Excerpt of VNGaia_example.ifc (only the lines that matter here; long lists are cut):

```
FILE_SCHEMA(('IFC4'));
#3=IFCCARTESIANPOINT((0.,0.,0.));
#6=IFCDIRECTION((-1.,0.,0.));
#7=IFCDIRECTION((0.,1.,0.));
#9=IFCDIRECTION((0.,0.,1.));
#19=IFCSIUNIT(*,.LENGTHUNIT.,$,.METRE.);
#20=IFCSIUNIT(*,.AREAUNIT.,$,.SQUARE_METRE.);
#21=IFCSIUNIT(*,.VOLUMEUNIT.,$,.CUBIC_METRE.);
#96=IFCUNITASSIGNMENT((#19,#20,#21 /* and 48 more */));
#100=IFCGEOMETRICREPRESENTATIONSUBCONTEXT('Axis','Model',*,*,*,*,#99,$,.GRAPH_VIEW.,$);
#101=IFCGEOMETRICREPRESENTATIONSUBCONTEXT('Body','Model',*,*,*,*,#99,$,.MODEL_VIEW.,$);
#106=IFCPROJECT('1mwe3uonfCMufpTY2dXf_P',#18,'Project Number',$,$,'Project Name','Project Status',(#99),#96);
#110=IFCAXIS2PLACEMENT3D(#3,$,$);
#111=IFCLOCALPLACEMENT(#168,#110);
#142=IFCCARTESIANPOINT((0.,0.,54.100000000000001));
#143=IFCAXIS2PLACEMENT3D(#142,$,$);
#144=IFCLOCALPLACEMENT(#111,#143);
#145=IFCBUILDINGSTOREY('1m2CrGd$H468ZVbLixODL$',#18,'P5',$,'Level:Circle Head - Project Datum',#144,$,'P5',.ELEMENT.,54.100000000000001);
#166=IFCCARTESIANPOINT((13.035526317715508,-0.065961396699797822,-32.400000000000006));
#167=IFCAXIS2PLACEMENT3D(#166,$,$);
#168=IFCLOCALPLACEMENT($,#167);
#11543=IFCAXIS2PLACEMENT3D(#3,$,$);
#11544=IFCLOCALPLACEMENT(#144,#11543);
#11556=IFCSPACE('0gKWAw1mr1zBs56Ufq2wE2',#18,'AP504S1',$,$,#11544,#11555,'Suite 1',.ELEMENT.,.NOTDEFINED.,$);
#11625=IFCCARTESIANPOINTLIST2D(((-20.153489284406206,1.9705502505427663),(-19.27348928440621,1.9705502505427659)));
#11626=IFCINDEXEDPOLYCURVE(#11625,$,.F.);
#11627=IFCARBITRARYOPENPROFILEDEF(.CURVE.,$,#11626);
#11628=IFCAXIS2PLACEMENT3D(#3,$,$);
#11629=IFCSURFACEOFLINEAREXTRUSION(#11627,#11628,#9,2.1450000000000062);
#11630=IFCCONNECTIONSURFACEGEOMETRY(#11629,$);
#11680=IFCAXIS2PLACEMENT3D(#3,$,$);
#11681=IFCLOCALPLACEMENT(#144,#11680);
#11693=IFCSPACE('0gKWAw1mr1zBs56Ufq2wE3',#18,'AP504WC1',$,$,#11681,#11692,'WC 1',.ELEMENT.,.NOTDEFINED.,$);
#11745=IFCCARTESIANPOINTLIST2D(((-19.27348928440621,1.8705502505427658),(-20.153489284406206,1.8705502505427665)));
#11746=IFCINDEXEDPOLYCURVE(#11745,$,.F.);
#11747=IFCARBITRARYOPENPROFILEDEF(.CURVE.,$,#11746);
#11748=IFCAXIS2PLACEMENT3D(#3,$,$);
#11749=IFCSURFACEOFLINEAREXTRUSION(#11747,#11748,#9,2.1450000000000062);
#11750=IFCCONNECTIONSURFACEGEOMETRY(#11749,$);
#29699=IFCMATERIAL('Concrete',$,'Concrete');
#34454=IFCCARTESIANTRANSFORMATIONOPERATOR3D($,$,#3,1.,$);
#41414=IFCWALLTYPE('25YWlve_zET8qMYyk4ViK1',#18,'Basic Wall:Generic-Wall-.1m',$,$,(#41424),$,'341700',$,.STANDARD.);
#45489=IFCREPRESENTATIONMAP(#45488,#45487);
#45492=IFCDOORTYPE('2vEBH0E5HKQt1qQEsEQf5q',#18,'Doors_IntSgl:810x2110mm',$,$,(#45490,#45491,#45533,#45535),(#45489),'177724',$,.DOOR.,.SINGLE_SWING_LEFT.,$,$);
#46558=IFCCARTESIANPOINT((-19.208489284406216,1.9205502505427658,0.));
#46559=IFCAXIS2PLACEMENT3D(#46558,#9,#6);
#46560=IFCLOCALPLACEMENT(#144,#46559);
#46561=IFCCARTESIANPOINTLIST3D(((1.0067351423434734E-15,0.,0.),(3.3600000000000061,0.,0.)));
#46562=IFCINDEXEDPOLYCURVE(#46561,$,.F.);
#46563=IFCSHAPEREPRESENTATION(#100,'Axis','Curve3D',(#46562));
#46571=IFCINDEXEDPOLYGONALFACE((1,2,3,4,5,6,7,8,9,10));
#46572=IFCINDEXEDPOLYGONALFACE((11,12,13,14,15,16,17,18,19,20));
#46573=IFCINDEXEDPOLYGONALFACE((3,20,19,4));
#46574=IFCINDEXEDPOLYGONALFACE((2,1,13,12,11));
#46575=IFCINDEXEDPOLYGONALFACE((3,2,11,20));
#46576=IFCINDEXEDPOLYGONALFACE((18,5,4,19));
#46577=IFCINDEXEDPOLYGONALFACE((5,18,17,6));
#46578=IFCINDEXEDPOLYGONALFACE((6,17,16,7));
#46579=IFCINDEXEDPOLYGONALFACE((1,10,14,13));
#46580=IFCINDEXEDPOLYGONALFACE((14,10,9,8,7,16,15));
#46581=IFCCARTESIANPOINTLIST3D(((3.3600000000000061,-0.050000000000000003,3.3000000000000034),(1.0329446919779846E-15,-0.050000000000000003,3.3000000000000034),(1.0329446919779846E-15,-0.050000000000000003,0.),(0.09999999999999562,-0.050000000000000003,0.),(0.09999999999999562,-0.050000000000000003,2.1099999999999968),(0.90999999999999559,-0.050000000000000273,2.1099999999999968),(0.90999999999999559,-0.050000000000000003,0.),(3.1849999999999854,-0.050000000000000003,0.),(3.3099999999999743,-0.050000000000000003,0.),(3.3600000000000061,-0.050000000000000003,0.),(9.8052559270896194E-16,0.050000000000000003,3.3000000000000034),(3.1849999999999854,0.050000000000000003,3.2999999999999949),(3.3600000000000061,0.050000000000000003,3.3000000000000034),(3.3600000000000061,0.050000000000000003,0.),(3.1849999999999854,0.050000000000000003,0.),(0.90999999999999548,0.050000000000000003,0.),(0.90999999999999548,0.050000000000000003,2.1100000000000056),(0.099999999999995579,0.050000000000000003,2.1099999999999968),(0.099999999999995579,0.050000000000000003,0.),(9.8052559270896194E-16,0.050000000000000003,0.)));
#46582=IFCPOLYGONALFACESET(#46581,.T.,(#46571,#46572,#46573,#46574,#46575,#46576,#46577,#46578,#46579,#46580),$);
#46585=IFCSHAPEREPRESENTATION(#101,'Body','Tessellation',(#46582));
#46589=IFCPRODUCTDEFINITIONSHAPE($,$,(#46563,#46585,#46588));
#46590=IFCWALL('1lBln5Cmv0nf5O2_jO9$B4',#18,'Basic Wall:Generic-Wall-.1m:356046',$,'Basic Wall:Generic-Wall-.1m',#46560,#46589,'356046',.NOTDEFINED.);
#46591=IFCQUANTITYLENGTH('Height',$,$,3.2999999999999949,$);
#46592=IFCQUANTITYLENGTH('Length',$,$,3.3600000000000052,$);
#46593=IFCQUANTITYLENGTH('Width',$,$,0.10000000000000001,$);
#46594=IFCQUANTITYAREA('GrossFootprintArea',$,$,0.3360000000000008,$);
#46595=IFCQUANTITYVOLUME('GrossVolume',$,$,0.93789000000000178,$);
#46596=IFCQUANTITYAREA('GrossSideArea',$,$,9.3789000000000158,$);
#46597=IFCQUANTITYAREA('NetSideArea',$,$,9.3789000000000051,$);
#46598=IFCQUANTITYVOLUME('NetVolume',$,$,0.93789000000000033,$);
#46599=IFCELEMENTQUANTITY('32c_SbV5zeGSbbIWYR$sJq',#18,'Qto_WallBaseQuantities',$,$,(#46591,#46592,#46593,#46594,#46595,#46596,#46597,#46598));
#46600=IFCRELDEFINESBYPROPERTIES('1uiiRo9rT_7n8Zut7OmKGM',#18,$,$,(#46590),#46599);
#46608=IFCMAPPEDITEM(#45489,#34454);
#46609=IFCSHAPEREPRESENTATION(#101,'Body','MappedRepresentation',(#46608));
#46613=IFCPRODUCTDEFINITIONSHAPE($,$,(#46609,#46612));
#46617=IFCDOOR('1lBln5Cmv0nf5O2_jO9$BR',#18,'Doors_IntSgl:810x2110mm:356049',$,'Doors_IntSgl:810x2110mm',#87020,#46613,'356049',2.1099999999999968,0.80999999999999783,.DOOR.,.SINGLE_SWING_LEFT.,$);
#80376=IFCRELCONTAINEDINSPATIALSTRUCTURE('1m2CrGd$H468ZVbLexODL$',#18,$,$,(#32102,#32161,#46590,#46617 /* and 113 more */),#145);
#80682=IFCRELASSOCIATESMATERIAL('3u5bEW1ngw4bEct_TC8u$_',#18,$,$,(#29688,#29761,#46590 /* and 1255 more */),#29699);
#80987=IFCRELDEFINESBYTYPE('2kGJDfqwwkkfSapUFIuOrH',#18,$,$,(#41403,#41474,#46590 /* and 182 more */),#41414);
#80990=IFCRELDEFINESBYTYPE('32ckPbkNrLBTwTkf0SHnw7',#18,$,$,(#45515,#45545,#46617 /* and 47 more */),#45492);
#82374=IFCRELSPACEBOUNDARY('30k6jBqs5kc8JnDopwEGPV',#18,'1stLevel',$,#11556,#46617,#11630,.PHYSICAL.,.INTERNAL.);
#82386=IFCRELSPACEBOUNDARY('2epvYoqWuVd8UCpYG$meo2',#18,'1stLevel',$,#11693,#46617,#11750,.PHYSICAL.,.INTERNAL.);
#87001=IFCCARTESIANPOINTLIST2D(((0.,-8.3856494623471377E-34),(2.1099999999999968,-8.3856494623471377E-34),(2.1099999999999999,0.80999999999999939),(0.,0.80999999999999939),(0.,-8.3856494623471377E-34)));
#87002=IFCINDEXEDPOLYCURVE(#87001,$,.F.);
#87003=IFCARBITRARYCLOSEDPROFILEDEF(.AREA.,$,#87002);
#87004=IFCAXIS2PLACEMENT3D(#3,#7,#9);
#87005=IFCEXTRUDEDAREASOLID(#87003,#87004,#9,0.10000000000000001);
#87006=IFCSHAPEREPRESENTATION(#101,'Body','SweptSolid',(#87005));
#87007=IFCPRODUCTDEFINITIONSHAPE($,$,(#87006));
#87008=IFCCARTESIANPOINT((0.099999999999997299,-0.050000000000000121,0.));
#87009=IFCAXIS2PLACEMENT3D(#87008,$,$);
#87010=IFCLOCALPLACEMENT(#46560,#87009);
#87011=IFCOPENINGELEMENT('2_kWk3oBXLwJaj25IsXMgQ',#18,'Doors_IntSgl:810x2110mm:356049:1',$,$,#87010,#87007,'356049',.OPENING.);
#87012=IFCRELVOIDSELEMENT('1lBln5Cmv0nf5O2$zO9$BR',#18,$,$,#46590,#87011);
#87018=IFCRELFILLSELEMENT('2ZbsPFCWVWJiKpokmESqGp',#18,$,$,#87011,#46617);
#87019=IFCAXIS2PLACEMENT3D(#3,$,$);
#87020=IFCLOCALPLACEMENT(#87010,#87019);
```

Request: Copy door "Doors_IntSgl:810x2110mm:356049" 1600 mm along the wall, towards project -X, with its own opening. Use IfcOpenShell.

```python
import numpy as np
import ifcopenshell
import ifcopenshell.api.feature
import ifcopenshell.api.geometry
import ifcopenshell.api.pset
import ifcopenshell.api.root
import ifcopenshell.geom
import ifcopenshell.util.element
import ifcopenshell.util.placement
import ifcopenshell.util.shape
import ifcopenshell.util.unit

model = ifcopenshell.open("VNGaia_example.ifc")
area_scale = ifcopenshell.util.unit.calculate_unit_scale(model, "AREAUNIT")
volume_scale = ifcopenshell.util.unit.calculate_unit_scale(model, "VOLUMEUNIT")
settings = ifcopenshell.geom.settings()


def volume(element):
    """Net volume in cubic metres, openings subtracted."""
    shape = ifcopenshell.geom.create_shape(settings, element)
    return ifcopenshell.util.shape.get_volume(shape.geometry)


def reuse_history(source, copy):
    """copy_class also copies each property set's owner history, people and application; keep the originals."""
    for rel in copy.IsDefinedBy:
        if rel.is_a("IfcRelDefinesByProperties") and (history := rel.RelatingPropertyDefinition.OwnerHistory):
            rel.RelatingPropertyDefinition.OwnerHistory = source.OwnerHistory
            ifcopenshell.util.element.remove_deep2(model, history)


door = model.by_guid("1lBln5Cmv0nf5O2_jO9$BR")
opening = door.FillsVoids[0].RelatingOpeningElement
wall = opening.VoidsElements[0].RelatingBuildingElement
before = volume(wall)
shift = ifcopenshell.util.placement.get_local_placement(wall.ObjectPlacement)[:3, 0] * 1.6

# copy_class copies the void relationship, type, container and properties, but no geometry.
new_opening = ifcopenshell.api.root.copy_class(model, product=opening)
new_opening.Representation = ifcopenshell.util.element.copy_deep(
    model, opening.Representation, exclude=["IfcGeometricRepresentationContext", "IfcRepresentationMap"]
)
new_opening.Name = "Doors_IntSgl:810x2110mm"
new_opening.Tag = None
reuse_history(opening, new_opening)
new_door = ifcopenshell.api.root.copy_class(model, product=door)
new_door.Representation = ifcopenshell.util.element.copy_deep(
    model, door.Representation, exclude=["IfcGeometricRepresentationContext", "IfcRepresentationMap"]
)
new_door.Name = "Doors_IntSgl:810x2110mm"
new_door.Tag = None
reuse_history(door, new_door)
ifcopenshell.api.feature.add_filling(model, opening=new_opening, element=new_door)

for old, new in ((opening, new_opening), (door, new_door)):
    matrix = ifcopenshell.util.placement.get_local_placement(old.ObjectPlacement)
    matrix[:3, 3] += shift
    ifcopenshell.api.geometry.edit_object_placement(model, product=new, matrix=matrix, is_si=False)

# The copied space boundaries still share their surfaces with the original.
for rel in new_door.ProvidesBoundaries:
    if rel.ConnectionGeometry:
        rel.ConnectionGeometry = ifcopenshell.util.element.copy_deep(model, rel.ConnectionGeometry)

# Space boundary surfaces are stored in each space's coordinates; move them too.
for rel in new_door.ProvidesBoundaries:
    if not rel.ConnectionGeometry:
        continue
    surface = rel.ConnectionGeometry.SurfaceOnRelatingElement
    space_matrix = ifcopenshell.util.placement.get_local_placement(rel.RelatingSpace.ObjectPlacement)
    point = np.array(surface.Position.Location.Coordinates) + space_matrix[:3, :3].T @ shift
    surface.Position = model.createIfcAxis2Placement3D(
        model.createIfcCartesianPoint(point.tolist()), surface.Position.Axis, surface.Position.RefDirection
    )

after = volume(wall)
thickness = 0.1  # wall thickness in metres

# Update the wall's stored quantities.
qto = model.by_id(ifcopenshell.util.element.get_pset(wall, "Qto_WallBaseQuantities", should_inherit=False)["id"])
ifcopenshell.api.pset.edit_qto(model, qto=qto, properties={
    "NetSideArea": after / thickness / area_scale,
    "NetVolume": after / volume_scale,
})

print(f"wall volume {before:.3f} -> {after:.3f} m3")

model.write("VNGaia_example_v2.ifc")
```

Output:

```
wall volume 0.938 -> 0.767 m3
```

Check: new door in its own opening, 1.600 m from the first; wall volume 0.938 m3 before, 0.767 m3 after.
